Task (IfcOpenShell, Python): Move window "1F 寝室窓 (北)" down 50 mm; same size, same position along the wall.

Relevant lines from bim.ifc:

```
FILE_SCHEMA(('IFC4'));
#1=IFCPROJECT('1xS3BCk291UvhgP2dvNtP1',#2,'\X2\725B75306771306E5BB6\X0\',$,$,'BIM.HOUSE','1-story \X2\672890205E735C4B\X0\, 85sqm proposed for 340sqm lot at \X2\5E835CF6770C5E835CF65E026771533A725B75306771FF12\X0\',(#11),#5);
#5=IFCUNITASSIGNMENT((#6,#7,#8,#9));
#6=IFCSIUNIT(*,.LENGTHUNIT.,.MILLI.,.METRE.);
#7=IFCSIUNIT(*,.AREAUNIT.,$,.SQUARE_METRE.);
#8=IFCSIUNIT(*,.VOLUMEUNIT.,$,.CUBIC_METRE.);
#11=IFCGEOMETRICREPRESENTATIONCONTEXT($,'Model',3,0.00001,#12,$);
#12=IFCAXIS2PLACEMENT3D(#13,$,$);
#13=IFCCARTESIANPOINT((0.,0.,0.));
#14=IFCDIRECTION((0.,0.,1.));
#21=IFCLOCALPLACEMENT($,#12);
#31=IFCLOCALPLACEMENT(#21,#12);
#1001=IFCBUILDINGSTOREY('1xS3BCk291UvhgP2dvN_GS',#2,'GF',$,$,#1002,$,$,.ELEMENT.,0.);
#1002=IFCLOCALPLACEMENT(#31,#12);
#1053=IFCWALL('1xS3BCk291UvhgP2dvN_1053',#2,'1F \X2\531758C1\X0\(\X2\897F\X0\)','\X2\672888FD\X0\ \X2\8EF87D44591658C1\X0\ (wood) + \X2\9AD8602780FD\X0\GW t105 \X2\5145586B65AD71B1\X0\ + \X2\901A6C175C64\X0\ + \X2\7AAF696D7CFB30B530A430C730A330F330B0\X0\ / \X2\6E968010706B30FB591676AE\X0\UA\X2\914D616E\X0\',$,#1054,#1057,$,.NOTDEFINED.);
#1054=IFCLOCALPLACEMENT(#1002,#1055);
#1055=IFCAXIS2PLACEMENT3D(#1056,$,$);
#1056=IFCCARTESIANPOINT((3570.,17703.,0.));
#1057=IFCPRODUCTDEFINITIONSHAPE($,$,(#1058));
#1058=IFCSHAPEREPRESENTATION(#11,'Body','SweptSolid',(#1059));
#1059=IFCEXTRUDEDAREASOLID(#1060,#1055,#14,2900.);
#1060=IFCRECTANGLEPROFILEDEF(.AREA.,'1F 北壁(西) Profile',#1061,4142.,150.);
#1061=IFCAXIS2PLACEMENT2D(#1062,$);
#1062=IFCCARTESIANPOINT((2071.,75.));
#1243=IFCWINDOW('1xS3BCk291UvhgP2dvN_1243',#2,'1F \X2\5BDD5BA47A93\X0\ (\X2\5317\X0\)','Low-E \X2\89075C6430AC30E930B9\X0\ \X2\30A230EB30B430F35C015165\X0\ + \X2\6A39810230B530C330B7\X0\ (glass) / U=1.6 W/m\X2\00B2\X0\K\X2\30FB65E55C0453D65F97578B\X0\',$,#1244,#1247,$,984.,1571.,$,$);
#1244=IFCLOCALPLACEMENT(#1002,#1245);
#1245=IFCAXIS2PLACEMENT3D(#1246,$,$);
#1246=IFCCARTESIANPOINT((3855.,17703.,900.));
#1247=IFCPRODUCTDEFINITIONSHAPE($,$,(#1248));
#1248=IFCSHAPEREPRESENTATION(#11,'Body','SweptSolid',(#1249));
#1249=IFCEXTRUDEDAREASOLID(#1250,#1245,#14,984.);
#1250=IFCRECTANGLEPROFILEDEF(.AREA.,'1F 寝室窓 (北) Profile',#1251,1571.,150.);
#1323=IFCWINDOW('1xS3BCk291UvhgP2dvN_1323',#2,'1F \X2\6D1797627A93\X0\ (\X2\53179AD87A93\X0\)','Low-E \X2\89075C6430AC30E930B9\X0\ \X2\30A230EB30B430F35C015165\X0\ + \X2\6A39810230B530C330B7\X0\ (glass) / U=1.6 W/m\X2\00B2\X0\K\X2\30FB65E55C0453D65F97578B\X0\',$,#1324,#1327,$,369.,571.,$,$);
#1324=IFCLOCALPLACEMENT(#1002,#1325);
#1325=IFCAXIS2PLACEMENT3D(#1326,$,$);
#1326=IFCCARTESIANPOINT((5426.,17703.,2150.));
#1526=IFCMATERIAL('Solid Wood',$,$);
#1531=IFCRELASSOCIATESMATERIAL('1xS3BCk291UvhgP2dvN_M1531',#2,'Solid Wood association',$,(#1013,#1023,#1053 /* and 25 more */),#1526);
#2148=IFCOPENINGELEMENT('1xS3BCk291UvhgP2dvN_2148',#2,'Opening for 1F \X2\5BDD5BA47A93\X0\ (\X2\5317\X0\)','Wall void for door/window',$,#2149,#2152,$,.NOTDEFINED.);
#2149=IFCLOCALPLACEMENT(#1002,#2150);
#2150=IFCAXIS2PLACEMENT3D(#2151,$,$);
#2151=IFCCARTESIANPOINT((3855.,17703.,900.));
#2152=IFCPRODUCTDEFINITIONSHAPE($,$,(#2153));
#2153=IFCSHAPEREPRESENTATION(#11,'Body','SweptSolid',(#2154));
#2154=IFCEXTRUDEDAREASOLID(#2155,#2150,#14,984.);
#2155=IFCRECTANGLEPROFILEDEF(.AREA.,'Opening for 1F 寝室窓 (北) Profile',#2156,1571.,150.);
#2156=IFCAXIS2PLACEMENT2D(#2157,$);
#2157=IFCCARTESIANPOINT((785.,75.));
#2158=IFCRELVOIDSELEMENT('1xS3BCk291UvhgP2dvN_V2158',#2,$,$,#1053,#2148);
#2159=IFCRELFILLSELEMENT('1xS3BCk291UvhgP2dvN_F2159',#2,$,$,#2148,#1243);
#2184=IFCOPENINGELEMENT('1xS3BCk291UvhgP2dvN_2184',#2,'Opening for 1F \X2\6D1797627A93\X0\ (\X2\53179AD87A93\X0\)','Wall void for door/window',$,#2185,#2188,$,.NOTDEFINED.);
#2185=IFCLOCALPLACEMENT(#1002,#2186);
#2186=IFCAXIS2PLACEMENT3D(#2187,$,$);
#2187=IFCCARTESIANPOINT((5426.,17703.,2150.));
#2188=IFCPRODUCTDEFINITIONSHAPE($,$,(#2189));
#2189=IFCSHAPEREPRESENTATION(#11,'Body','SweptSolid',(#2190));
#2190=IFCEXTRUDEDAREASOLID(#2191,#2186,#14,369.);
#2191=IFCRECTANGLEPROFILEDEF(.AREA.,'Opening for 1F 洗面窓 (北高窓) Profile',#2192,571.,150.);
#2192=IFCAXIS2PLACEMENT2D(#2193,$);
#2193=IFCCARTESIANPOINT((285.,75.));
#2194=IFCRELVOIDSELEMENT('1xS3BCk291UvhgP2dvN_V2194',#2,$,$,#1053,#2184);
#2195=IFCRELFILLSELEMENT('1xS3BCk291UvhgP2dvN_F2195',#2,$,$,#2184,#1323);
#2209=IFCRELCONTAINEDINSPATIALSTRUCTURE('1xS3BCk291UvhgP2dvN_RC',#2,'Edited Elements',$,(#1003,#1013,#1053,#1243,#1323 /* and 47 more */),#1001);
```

```python
import numpy as np
import ifcopenshell
import ifcopenshell.api.geometry
import ifcopenshell.util.placement
import ifcopenshell.util.unit

model = ifcopenshell.open("bim.ifc")
unit_scale = ifcopenshell.util.unit.calculate_unit_scale(model)

window = model.by_id(1243)
opening = window.FillsVoids[0].RelatingOpeningElement
dz = -0.05 / unit_scale

shift = np.array([0.0, 0.0, dz])
# The window is not placed relative to its opening, so move both.
for product in (opening, window):
    matrix = ifcopenshell.util.placement.get_local_placement(product.ObjectPlacement)
    matrix[:3, 3] += shift
    ifcopenshell.api.geometry.edit_object_placement(model, product=product, matrix=matrix, is_si=False)

print(f"moved by {dz * unit_scale:+.3f} m")

model.write("bim_v2.ifc")
```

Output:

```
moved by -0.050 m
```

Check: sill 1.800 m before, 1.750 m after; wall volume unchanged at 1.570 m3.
